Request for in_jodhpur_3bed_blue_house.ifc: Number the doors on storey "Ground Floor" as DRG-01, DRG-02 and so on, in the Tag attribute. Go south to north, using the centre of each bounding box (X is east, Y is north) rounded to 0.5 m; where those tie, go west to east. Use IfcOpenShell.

First a look at what the model holds.

```python
import ifcopenshell
import ifcopenshell.util.element
import ifcopenshell.util.placement

model = ifcopenshell.open("in_jodhpur_3bed_blue_house.ifc")
print(model.schema)
storey = next(s for s in model.by_type("IfcBuildingStorey") if s.Name == "Ground Floor")
doors = [e for e in ifcopenshell.util.element.get_decomposition(storey) if e.is_a("IfcDoor")]
for e in sorted(doors, key=lambda e: e.id()):
    origin = ifcopenshell.util.placement.get_local_placement(e.ObjectPlacement)[:3, 3]
    print(e.id(), e.Tag, e.Name, origin.round(2) + 0.0, sep=" | ")
```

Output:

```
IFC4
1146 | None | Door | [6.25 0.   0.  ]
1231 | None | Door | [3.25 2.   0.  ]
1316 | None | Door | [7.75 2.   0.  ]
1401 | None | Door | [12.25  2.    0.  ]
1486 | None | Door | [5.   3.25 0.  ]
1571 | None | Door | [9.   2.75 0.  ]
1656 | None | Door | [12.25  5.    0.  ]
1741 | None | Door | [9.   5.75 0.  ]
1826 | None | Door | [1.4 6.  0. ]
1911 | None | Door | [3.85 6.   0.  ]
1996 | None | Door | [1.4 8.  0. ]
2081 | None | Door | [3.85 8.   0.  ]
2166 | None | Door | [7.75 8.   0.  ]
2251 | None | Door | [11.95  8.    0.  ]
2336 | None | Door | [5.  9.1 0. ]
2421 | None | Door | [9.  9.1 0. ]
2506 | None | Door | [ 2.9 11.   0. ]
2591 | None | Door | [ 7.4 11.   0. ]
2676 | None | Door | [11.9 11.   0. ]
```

```python
import ifcopenshell
import ifcopenshell.geom
import ifcopenshell.util.element
import ifcopenshell.util.shape

model = ifcopenshell.open("in_jodhpur_3bed_blue_house.ifc")
settings = ifcopenshell.geom.settings()
settings.set("use-world-coords", True)


def centre(element):
    shape = ifcopenshell.geom.create_shape(settings, element)
    return ifcopenshell.util.shape.get_bbox_centroid(shape.geometry)


storey = next(s for s in model.by_type("IfcBuildingStorey") if s.Name == "Ground Floor")
doors = [e for e in ifcopenshell.util.element.get_decomposition(storey) if e.is_a("IfcDoor")]

# Insertion points can sit at a corner or the storey origin, so sort by the geometry (in metres).
centres = {e: centre(e) for e in doors}
doors.sort(key=lambda e: (round(centres[e][1] / 0.5), centres[e][0]))

for i, e in enumerate(doors, start=1):
    number = f"DRG-{i:02d}"
    e.Tag = number
    print(e.id(), number)

model.write("in_jodhpur_3bed_blue_house_edited.ifc")
```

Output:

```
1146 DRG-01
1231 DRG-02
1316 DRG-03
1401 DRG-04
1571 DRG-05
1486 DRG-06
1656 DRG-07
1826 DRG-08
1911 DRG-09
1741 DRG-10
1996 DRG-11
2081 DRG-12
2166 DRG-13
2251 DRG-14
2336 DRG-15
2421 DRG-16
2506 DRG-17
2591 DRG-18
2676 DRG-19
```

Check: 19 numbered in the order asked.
